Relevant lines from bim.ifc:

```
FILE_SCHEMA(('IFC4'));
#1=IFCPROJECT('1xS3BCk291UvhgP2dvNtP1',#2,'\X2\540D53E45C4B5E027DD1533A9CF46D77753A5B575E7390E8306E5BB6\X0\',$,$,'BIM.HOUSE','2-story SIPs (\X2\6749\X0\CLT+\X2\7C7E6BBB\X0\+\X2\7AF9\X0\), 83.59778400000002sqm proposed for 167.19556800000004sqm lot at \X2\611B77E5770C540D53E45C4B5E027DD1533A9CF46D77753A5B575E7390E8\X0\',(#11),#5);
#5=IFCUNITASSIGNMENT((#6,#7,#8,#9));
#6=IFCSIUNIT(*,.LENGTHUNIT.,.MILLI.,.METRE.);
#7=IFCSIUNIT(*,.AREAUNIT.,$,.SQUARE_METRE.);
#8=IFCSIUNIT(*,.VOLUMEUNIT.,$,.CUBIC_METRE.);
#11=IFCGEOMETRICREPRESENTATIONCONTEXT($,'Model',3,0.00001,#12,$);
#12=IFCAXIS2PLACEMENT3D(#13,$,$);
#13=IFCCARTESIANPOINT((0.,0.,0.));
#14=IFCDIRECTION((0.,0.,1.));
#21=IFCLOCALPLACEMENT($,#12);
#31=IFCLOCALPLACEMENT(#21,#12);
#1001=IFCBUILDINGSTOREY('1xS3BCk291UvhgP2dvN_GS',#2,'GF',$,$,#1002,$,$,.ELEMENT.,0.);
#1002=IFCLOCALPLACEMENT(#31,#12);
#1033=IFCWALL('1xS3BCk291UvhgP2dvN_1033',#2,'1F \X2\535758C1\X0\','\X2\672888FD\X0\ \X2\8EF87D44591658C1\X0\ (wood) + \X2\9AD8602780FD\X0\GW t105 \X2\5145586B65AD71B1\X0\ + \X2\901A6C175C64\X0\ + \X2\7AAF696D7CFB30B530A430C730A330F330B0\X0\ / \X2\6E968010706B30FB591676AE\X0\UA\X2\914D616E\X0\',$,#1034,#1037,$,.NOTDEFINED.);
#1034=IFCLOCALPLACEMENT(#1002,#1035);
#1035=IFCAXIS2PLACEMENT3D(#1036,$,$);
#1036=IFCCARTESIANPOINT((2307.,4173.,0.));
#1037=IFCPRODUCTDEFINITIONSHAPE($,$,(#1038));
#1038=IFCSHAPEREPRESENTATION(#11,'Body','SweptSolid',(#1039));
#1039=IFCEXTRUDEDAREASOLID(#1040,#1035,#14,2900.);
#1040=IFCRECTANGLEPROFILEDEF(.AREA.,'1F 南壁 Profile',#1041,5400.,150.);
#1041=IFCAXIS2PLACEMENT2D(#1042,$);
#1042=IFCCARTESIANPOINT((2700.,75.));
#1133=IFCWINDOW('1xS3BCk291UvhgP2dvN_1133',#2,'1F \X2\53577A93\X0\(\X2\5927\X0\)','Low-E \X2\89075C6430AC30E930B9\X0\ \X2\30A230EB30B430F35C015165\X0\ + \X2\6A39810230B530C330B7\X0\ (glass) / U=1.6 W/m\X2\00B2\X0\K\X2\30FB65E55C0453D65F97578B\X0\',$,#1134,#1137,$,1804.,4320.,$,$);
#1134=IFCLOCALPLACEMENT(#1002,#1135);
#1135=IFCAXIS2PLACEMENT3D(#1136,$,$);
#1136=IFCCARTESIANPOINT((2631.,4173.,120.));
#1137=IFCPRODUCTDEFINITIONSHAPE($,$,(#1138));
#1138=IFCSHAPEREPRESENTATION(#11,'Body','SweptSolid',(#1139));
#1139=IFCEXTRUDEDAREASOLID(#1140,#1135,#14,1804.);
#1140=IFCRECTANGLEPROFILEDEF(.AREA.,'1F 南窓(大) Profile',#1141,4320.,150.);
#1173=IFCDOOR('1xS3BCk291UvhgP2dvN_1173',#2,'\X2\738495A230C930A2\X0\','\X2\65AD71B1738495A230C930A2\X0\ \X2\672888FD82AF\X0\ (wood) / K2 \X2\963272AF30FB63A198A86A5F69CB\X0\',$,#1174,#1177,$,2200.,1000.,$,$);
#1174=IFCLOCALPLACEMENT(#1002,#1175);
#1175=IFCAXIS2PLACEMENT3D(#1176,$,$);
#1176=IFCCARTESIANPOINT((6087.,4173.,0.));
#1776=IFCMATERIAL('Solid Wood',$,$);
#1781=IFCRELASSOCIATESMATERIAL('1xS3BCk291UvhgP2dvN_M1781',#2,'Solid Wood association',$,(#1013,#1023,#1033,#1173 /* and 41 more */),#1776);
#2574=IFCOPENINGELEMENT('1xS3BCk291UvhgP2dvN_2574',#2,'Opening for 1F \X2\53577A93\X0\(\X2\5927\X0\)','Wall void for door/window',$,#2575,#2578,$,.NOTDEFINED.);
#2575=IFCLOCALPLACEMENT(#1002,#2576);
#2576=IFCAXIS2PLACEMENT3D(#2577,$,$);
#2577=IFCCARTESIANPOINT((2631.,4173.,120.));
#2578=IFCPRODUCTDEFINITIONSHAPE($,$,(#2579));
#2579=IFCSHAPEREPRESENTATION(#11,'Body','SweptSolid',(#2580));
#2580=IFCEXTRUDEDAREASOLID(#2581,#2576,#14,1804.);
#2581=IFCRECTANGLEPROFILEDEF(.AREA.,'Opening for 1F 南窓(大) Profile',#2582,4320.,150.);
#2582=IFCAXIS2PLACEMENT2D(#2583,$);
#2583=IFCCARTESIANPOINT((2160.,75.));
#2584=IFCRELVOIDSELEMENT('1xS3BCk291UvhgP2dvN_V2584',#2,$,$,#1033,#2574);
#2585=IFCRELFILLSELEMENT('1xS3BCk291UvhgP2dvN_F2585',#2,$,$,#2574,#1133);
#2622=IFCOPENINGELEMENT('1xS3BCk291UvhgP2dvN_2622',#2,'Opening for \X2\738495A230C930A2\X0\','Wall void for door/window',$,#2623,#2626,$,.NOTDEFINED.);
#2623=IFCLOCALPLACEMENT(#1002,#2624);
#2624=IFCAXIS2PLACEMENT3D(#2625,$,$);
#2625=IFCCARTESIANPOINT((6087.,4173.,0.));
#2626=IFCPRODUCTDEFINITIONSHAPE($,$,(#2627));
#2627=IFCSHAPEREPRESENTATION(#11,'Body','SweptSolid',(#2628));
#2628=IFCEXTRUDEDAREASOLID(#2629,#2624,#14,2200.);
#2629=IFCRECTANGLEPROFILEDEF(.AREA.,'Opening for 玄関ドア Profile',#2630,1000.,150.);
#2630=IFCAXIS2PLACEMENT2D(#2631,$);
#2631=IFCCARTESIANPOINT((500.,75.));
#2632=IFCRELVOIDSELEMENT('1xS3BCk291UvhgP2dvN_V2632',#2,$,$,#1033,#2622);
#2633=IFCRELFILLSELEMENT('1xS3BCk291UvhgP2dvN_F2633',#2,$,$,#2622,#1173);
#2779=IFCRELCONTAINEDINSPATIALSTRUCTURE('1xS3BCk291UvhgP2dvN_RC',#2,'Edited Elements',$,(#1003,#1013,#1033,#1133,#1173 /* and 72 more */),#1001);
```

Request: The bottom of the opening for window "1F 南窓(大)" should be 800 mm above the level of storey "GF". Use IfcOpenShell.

```python
import numpy as np
import ifcopenshell
import ifcopenshell.api.geometry
import ifcopenshell.geom
import ifcopenshell.util.element
import ifcopenshell.util.placement
import ifcopenshell.util.shape
import ifcopenshell.util.unit

model = ifcopenshell.open("bim.ifc")
unit_scale = ifcopenshell.util.unit.calculate_unit_scale(model)

window = model.by_guid("1xS3BCk291UvhgP2dvN_1133")
opening = window.FillsVoids[0].RelatingOpeningElement
storey = ifcopenshell.util.element.get_container(window, ifc_class="IfcBuildingStorey")
level = ifcopenshell.util.placement.get_local_placement(storey.ObjectPlacement)[2, 3]

# The opening's origin need not be at the sill, so measure its lowest point.
shape = ifcopenshell.geom.create_shape(ifcopenshell.geom.settings(), opening)
bottom = ifcopenshell.util.shape.get_shape_bottom_elevation(shape, shape.geometry) / unit_scale
dz = level + 0.8 / unit_scale - bottom

shift = np.array([0.0, 0.0, dz])
# The window is not placed relative to its opening, so move both.
for product in (opening, window):
    matrix = ifcopenshell.util.placement.get_local_placement(product.ObjectPlacement)
    matrix[:3, 3] += shift
    ifcopenshell.api.geometry.edit_object_placement(model, product=product, matrix=matrix, is_si=False)

print(f"moved by {dz * unit_scale:+.3f} m")

model.write("bim_edited.ifc")
```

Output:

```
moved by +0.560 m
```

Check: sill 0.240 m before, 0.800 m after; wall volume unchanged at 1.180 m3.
